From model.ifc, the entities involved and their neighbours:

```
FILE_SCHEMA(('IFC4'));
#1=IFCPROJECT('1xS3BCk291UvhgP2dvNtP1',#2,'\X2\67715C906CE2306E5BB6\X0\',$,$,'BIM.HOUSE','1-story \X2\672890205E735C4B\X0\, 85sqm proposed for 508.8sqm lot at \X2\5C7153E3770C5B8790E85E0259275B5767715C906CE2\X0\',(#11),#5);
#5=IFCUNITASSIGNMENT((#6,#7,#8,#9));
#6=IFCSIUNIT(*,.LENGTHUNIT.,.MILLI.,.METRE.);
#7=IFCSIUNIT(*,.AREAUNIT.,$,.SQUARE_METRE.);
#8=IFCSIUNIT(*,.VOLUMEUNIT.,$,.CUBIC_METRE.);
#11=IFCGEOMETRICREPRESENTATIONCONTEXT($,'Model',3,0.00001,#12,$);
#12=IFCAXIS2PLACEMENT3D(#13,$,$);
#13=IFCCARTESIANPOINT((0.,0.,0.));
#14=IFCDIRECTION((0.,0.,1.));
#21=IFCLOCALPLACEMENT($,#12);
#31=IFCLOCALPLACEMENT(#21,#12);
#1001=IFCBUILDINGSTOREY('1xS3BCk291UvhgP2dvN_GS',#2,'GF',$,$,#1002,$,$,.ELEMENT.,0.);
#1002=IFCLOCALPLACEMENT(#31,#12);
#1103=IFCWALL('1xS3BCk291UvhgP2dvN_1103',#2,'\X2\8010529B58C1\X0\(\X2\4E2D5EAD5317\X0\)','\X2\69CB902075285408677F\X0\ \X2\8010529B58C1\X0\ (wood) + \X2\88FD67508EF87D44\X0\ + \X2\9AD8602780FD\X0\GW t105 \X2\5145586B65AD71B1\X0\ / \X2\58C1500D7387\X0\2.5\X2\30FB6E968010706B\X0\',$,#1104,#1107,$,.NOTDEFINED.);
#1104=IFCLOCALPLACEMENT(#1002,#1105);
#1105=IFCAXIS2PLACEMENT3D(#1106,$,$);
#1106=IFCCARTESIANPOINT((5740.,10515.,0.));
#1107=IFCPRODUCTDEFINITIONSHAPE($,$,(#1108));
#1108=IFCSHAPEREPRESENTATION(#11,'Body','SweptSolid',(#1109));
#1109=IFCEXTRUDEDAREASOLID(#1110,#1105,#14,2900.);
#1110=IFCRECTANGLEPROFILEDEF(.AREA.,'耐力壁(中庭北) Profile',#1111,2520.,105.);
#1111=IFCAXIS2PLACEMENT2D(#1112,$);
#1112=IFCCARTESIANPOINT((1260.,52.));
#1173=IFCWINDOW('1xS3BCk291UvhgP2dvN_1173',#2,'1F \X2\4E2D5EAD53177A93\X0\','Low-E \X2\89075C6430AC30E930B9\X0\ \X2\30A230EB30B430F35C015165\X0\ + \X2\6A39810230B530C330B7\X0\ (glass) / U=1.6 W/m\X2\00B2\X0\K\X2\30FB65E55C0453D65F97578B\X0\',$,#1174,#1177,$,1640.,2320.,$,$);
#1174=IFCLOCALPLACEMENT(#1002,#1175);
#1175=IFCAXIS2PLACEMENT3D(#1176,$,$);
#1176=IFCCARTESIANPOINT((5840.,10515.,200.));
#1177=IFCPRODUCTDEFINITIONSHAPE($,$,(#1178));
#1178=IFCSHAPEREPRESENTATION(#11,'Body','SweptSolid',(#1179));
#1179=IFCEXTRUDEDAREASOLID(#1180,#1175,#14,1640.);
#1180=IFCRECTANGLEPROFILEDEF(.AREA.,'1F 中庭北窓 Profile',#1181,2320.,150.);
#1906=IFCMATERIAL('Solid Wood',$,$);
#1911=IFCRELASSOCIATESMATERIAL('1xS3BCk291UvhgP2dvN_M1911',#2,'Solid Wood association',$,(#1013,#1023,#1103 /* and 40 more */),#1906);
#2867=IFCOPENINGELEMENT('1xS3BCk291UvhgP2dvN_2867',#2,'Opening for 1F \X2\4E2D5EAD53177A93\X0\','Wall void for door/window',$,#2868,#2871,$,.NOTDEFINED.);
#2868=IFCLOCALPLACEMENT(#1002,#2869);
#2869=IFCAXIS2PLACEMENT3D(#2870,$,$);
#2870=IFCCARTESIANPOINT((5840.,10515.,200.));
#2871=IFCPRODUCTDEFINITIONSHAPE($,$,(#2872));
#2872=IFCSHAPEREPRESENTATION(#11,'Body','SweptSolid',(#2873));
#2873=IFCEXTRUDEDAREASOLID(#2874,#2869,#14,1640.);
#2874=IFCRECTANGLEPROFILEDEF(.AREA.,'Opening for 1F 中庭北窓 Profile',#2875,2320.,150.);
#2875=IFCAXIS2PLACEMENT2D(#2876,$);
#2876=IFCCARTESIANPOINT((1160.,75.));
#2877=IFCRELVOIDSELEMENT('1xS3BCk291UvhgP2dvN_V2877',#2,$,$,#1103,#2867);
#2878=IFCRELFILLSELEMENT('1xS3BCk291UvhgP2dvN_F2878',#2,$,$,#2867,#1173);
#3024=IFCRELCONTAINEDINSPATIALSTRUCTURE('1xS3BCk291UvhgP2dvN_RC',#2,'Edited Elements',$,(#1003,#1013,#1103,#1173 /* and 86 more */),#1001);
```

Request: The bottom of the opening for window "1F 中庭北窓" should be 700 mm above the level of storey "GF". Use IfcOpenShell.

```python
import numpy as np
import ifcopenshell
import ifcopenshell.api.geometry
import ifcopenshell.geom
import ifcopenshell.util.element
import ifcopenshell.util.placement
import ifcopenshell.util.shape
import ifcopenshell.util.unit

model = ifcopenshell.open("model.ifc")
unit_scale = ifcopenshell.util.unit.calculate_unit_scale(model)

window = model.by_guid("1xS3BCk291UvhgP2dvN_1173")
opening = window.FillsVoids[0].RelatingOpeningElement
storey = ifcopenshell.util.element.get_container(window, ifc_class="IfcBuildingStorey")
level = ifcopenshell.util.placement.get_local_placement(storey.ObjectPlacement)[2, 3]

# The opening's origin need not be at the sill, so measure its lowest point.
shape = ifcopenshell.geom.create_shape(ifcopenshell.geom.settings(), opening)
bottom = ifcopenshell.util.shape.get_shape_bottom_elevation(shape, shape.geometry) / unit_scale
dz = level + 700.0 - bottom

shift = np.array([0.0, 0.0, dz])
# The window is not placed relative to its opening, so move both.
for product in (opening, window):
    matrix = ifcopenshell.util.placement.get_local_placement(product.ObjectPlacement)
    matrix[:3, 3] += shift
    ifcopenshell.api.geometry.edit_object_placement(model, product=product, matrix=matrix, is_si=False)

print(f"moved by {dz * unit_scale:+.3f} m")

model.write("model-out.ifc")
```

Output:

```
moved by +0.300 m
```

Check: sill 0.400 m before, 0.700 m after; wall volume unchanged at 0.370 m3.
